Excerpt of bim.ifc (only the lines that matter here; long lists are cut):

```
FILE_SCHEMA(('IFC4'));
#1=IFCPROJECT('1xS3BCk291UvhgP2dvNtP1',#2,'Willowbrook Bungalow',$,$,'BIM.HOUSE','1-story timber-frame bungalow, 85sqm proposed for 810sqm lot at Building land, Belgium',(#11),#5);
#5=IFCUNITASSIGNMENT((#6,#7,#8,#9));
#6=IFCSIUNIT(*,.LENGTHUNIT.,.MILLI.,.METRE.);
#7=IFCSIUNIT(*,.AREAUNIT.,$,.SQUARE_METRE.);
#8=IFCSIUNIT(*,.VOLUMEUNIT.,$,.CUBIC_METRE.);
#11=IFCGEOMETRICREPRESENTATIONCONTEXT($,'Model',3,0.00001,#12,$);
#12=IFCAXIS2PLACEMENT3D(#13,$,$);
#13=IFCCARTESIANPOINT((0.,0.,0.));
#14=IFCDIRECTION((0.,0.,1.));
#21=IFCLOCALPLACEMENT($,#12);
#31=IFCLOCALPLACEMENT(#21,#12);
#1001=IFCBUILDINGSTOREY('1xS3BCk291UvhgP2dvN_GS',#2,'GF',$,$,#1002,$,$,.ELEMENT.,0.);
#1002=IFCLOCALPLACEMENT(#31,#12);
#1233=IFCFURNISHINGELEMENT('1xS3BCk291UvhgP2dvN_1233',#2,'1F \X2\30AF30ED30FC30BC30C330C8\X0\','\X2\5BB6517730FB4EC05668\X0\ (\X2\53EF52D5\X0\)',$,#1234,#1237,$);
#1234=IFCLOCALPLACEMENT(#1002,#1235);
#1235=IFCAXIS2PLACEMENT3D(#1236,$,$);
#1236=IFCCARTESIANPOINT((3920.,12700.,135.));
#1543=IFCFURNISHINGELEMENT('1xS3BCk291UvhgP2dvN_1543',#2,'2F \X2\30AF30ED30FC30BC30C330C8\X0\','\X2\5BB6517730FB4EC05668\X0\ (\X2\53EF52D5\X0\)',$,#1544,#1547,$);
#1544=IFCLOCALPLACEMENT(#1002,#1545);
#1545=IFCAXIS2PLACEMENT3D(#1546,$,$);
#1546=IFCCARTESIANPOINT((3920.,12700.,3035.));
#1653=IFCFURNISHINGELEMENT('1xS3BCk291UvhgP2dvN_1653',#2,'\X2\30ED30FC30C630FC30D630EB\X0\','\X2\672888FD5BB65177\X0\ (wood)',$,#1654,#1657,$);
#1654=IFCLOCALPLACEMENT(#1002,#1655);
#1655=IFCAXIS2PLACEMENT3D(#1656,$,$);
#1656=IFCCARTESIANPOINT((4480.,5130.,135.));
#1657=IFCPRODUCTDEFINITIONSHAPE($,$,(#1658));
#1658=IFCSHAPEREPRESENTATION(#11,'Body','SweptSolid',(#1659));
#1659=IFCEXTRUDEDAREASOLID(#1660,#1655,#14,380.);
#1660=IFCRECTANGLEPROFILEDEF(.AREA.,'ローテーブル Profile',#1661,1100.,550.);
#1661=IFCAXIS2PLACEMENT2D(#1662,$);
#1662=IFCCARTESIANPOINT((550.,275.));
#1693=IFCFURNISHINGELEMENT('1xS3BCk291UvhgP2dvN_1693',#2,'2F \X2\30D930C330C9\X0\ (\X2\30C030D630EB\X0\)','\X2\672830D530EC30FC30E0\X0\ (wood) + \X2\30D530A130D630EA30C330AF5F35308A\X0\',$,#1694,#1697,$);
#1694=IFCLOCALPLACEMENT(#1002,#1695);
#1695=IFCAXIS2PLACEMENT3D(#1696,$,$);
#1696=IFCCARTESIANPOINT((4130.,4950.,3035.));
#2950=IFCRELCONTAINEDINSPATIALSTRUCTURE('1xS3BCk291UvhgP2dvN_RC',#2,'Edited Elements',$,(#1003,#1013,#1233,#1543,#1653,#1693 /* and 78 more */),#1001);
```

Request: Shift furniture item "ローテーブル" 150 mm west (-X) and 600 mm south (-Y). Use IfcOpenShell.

```python
import ifcopenshell
import ifcopenshell.api.geometry
import ifcopenshell.util.placement
import ifcopenshell.util.unit

model = ifcopenshell.open("bim.ifc")
unit_scale = ifcopenshell.util.unit.calculate_unit_scale(model)

item = model.by_guid("1xS3BCk291UvhgP2dvN_1653")
matrix = ifcopenshell.util.placement.get_local_placement(item.ObjectPlacement)
matrix[0, 3] -= 0.15 / unit_scale
matrix[1, 3] -= 0.6 / unit_scale
ifcopenshell.api.geometry.edit_object_placement(model, product=item, matrix=matrix, is_si=False)

print(ifcopenshell.util.placement.get_local_placement(item.ObjectPlacement).round(3) + 0.0)

model.write("bim_updated.ifc")
```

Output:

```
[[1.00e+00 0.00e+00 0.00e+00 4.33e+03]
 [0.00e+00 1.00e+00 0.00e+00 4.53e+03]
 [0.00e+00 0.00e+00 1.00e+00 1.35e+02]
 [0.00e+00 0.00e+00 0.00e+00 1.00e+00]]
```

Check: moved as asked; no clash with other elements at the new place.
